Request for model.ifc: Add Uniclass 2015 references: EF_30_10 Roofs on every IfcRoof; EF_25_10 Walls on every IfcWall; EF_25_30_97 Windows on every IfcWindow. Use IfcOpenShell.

First a look at what the model holds.

```python
import ifcopenshell

model = ifcopenshell.open("model.ifc")
print(model.schema)
print("classifications:", [c.Name for c in model.by_type("IfcClassification")])
for ifc_class in ("IfcDoor", "IfcRoof", "IfcStair", "IfcWall", "IfcWindow"):
    print(ifc_class, len(model.by_type(ifc_class)))
```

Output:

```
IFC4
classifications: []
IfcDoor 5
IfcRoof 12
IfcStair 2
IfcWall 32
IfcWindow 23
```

```python
import ifcopenshell
import ifcopenshell.api.classification

model = ifcopenshell.open("model.ifc")

system = ifcopenshell.api.classification.add_classification(model, classification="Uniclass 2015")

codes = {
    "IfcRoof": ("EF_30_10", "Roofs"),
    "IfcWall": ("EF_25_10", "Walls"),
    "IfcWindow": ("EF_25_30_97", "Windows"),
}
for ifc_class, (code, name) in codes.items():
    products = model.by_type(ifc_class)
    ifcopenshell.api.classification.add_reference(
        model, products=products, classification=system, identification=code, name=name
    )
    print(code, len(products))

model.write("model_v2.ifc")
```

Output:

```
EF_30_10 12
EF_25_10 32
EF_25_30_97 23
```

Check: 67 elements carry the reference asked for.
